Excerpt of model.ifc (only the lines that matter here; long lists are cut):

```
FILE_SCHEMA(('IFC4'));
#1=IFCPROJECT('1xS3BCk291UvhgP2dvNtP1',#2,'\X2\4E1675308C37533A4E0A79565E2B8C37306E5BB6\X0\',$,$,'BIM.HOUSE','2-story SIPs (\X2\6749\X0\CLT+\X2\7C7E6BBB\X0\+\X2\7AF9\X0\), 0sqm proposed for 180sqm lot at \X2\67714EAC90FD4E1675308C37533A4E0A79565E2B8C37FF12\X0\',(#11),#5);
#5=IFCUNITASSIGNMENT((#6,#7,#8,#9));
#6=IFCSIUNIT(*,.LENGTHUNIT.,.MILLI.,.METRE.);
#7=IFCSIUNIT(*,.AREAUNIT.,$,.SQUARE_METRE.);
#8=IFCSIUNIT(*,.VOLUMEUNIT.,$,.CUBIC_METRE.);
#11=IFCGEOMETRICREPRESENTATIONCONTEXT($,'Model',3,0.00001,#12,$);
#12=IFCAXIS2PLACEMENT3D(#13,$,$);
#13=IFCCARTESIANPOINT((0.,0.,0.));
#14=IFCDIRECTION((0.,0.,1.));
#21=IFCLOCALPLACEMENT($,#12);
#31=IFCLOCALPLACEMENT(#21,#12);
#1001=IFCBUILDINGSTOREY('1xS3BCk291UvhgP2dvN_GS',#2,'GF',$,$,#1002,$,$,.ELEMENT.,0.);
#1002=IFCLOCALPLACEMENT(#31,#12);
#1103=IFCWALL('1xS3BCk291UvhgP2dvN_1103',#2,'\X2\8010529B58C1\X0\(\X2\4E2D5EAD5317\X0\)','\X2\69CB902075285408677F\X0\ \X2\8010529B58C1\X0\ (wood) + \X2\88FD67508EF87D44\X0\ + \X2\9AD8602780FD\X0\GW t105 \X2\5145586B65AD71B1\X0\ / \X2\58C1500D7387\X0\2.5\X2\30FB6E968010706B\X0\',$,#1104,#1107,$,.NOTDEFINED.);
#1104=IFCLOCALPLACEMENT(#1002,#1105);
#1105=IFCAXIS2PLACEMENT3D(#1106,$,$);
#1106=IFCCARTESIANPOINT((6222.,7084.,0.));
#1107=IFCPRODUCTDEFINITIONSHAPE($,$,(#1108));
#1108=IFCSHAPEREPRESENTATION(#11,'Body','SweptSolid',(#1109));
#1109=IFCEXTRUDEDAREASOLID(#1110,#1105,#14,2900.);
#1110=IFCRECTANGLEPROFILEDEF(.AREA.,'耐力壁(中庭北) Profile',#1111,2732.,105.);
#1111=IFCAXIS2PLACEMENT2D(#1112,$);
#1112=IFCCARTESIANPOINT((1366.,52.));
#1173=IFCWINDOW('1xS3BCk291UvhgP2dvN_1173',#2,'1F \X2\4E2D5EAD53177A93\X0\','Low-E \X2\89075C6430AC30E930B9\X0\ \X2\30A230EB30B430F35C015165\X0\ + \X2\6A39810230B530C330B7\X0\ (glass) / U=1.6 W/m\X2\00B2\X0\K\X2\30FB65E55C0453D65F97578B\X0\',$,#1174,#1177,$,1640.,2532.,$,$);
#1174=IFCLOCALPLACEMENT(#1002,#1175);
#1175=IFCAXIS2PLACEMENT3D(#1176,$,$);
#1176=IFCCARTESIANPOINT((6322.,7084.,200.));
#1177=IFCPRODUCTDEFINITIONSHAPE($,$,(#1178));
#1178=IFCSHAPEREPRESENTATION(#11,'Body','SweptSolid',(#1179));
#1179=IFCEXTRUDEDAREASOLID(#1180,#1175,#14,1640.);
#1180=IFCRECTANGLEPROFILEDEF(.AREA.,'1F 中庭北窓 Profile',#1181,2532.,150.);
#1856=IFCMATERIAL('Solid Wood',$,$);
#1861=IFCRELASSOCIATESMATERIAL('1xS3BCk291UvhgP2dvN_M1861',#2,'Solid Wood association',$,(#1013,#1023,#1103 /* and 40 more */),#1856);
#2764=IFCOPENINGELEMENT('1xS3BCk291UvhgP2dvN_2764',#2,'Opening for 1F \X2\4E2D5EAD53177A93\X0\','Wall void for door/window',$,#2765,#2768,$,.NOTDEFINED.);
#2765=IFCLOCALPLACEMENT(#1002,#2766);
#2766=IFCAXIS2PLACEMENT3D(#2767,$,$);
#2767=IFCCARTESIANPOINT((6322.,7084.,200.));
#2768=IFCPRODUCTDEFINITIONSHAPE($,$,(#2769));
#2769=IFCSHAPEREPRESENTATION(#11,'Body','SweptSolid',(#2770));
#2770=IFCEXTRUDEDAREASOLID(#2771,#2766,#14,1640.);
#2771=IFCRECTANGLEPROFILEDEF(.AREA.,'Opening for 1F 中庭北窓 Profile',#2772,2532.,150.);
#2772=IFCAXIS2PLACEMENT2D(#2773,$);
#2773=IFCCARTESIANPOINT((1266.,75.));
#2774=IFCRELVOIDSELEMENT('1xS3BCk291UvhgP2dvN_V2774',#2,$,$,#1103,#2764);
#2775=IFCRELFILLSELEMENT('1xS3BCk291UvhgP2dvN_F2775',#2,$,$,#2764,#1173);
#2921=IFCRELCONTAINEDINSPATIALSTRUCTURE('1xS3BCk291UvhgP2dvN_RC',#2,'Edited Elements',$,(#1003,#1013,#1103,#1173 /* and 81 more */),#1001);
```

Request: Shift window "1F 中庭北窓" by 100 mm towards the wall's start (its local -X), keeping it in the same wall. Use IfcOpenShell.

```python
import ifcopenshell
import ifcopenshell.api.geometry
import ifcopenshell.util.placement
import ifcopenshell.util.unit

model = ifcopenshell.open("model.ifc")
unit_scale = ifcopenshell.util.unit.calculate_unit_scale(model)

window = model.by_guid("1xS3BCk291UvhgP2dvN_1173")
opening = window.FillsVoids[0].RelatingOpeningElement
wall = opening.VoidsElements[0].RelatingBuildingElement

wall_matrix = ifcopenshell.util.placement.get_local_placement(wall.ObjectPlacement)
shift = wall_matrix[:3, 0] * -0.1 / unit_scale
before = ifcopenshell.util.placement.get_local_placement(window.ObjectPlacement)[:3, 3].copy()

# The window is not placed relative to its opening, so move both.
for product in (opening, window):
    matrix = ifcopenshell.util.placement.get_local_placement(product.ObjectPlacement)
    matrix[:3, 3] += shift
    ifcopenshell.api.geometry.edit_object_placement(model, product=product, matrix=matrix, is_si=False)

after = ifcopenshell.util.placement.get_local_placement(window.ObjectPlacement)[:3, 3]
print("window moved by", (after - before).round(3) + 0.0)

model.write("model_updated.ifc")
```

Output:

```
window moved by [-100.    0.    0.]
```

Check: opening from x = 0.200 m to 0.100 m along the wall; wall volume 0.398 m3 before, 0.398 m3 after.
